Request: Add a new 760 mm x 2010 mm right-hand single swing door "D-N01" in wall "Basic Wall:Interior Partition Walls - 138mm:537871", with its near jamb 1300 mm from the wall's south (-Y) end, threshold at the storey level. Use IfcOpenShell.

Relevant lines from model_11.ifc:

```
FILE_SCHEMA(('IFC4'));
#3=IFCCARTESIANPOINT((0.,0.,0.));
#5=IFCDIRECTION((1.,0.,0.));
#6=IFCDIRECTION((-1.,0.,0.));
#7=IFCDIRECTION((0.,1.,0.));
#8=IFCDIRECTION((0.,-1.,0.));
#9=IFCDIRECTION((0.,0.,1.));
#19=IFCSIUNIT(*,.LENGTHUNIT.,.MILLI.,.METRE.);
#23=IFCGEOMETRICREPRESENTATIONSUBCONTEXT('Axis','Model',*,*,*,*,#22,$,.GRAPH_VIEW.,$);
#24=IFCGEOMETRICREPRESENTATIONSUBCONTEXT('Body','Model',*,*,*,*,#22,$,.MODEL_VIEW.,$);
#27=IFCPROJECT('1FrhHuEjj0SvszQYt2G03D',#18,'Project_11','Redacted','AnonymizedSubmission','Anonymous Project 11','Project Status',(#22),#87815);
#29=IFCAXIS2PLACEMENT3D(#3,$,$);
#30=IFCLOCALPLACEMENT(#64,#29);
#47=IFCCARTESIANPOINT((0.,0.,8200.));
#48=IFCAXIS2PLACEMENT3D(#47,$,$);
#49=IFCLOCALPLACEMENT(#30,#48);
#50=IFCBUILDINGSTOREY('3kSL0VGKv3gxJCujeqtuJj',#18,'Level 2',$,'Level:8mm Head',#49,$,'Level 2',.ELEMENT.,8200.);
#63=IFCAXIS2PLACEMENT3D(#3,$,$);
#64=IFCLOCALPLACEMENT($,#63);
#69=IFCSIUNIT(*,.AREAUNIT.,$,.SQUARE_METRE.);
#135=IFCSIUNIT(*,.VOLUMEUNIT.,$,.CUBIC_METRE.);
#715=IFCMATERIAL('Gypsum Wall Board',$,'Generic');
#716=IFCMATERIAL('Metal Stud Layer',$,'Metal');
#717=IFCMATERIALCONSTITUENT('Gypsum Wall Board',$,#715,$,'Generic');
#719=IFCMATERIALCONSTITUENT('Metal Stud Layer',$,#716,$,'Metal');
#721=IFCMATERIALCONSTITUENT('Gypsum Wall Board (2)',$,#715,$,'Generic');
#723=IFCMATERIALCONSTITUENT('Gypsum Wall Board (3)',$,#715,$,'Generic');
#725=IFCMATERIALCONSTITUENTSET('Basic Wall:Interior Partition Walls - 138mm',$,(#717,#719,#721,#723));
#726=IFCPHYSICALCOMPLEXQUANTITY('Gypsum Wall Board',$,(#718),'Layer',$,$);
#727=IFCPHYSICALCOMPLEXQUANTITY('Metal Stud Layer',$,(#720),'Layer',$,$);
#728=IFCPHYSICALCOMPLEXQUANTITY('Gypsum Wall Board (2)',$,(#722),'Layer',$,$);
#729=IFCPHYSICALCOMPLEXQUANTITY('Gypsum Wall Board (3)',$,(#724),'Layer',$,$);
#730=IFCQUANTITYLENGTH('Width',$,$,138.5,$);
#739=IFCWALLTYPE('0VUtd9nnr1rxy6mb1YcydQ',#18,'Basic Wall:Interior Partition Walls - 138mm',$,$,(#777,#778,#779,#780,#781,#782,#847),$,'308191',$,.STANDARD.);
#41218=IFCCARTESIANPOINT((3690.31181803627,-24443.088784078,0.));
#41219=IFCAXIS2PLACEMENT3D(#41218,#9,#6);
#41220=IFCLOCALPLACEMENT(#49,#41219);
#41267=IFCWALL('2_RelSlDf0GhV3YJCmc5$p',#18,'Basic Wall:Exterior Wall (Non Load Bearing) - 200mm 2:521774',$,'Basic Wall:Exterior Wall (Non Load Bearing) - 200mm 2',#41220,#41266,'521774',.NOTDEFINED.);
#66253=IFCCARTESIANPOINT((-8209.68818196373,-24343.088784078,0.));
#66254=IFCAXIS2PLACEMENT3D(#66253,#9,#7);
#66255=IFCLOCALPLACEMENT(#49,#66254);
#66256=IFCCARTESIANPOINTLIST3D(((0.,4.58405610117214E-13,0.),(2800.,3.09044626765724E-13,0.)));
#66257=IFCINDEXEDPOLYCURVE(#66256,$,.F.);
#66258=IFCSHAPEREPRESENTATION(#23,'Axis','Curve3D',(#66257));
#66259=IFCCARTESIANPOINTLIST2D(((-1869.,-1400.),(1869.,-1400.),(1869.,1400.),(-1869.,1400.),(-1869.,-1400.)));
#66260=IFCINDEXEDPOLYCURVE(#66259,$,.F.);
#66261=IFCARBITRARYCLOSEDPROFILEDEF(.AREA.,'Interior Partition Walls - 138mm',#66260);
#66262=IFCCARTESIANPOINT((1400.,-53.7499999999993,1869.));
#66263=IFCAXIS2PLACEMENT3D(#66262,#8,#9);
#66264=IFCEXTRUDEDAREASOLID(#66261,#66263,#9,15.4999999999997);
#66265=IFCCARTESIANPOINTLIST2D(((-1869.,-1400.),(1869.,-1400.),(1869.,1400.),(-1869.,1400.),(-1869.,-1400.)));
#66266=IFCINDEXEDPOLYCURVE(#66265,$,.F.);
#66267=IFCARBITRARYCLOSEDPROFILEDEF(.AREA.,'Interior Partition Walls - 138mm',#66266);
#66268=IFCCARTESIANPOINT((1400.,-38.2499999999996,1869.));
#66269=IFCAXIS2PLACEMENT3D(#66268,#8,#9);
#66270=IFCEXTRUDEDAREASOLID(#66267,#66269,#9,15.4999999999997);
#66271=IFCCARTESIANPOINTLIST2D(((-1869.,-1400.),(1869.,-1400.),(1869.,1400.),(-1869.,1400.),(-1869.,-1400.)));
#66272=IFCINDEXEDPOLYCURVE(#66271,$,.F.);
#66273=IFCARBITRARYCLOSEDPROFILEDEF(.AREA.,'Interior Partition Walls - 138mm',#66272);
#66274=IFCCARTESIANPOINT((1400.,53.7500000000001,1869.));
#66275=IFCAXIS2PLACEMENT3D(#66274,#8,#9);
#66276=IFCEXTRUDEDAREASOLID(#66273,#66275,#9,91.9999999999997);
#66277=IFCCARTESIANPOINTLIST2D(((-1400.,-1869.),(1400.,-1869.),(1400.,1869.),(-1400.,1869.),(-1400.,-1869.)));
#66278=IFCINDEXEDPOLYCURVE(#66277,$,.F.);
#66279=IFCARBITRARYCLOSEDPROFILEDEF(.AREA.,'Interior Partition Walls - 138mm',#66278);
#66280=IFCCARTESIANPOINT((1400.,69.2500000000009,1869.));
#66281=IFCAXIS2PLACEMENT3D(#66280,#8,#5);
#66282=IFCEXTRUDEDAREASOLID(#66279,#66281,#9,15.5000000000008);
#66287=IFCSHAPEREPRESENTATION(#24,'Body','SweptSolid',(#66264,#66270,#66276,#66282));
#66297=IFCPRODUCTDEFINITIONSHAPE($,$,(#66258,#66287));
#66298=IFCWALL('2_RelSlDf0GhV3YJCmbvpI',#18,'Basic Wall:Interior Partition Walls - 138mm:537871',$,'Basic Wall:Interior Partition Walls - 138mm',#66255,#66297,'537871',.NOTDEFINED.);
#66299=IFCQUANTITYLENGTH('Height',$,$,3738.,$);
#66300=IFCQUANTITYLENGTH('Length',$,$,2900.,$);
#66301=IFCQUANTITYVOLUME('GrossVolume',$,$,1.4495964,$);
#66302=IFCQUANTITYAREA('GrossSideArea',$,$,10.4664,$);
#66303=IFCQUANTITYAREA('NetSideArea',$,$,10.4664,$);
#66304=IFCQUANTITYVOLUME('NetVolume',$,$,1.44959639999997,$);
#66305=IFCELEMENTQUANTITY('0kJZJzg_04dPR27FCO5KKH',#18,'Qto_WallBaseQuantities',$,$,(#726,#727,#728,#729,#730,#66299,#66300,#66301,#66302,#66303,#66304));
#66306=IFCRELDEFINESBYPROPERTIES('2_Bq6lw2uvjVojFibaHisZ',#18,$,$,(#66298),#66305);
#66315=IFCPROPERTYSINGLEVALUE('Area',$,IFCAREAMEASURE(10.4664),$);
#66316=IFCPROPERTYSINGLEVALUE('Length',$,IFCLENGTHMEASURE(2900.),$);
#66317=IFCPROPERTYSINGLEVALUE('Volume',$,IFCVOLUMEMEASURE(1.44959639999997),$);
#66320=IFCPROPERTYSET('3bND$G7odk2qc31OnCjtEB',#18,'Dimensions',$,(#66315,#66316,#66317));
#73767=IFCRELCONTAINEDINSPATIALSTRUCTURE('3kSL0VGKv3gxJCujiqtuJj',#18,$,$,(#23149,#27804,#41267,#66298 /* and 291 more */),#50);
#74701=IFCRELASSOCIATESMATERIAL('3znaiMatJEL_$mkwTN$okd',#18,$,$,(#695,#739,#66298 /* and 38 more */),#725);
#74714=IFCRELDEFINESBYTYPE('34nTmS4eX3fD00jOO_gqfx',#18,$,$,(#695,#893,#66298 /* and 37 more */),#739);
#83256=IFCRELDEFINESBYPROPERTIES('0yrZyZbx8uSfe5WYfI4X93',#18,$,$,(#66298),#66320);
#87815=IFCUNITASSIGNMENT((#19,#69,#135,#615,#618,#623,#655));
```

```python
import numpy as np
import ifcopenshell
import ifcopenshell.api.feature
import ifcopenshell.api.geometry
import ifcopenshell.api.pset
import ifcopenshell.api.root
import ifcopenshell.api.spatial
import ifcopenshell.geom
import ifcopenshell.util.element
import ifcopenshell.util.placement
import ifcopenshell.util.representation
import ifcopenshell.util.shape
import ifcopenshell.util.unit

model = ifcopenshell.open("model_11.ifc")
unit_scale = ifcopenshell.util.unit.calculate_unit_scale(model)
area_scale = ifcopenshell.util.unit.calculate_unit_scale(model, "AREAUNIT")
volume_scale = ifcopenshell.util.unit.calculate_unit_scale(model, "VOLUMEUNIT")
settings = ifcopenshell.geom.settings()


def volume(element):
    """Net volume in cubic metres, openings subtracted."""
    shape = ifcopenshell.geom.create_shape(settings, element)
    return ifcopenshell.util.shape.get_volume(shape.geometry)


wall = model.by_guid("2_RelSlDf0GhV3YJCmbvpI")
storey = ifcopenshell.util.element.get_container(wall, ifc_class="IfcBuildingStorey")
context = ifcopenshell.util.representation.get_context(model, "Model", "Body", "MODEL_VIEW")
before = volume(wall)

width, height, from_end, sill = 0.76, 2.01, 1.3, 0.0  # metres

# The wall runs along its own X axis, and the end named is its -X end.
wall_shape = ifcopenshell.geom.create_shape(settings, wall)
x, y, z = ifcopenshell.util.shape.get_vertices(wall_shape.geometry).T
start = x.min() + from_end
face, thickness = float(y.min()), float(y.max() - y.min())
wall_matrix = ifcopenshell.util.placement.get_local_placement(wall.ObjectPlacement)
level = ifcopenshell.util.placement.get_local_placement(storey.ObjectPlacement)[2, 3]


def in_wall(x, y):
    """Placement at x, y metres in the wall's axes, at sill height."""
    matrix = wall_matrix.copy()
    matrix[:, 3] = wall_matrix @ np.array([x / unit_scale, y / unit_scale, 0.0, 1.0])
    matrix[2, 3] = level + sill / unit_scale
    return matrix


# Opening: a box that overshoots both wall faces by 50 mm.
opening = ifcopenshell.api.root.create_entity(model, ifc_class="IfcOpeningElement", predefined_type="OPENING")
box = ifcopenshell.api.geometry.add_wall_representation(
    model, context=context, length=width, height=height, thickness=thickness + 0.1
)
ifcopenshell.api.geometry.assign_representation(model, product=opening, representation=box)
ifcopenshell.api.geometry.edit_object_placement(model, product=opening, matrix=in_wall(start, face - 0.05), is_si=False)
ifcopenshell.api.feature.add_feature(model, feature=opening, element=wall)

door = ifcopenshell.api.root.create_entity(model, ifc_class="IfcDoor", name="D-N01", predefined_type="DOOR")
door.OverallWidth, door.OverallHeight = width / unit_scale, height / unit_scale
door.OperationType = "SINGLE_SWING_RIGHT"
body = ifcopenshell.api.geometry.add_door_representation(
    model,
    context=context,
    overall_width=door.OverallWidth,
    overall_height=door.OverallHeight,
    operation_type="SINGLE_SWING_RIGHT",
    lining_properties={"LiningDepth": thickness / unit_scale, "ThresholdDepth": thickness / unit_scale},
)
ifcopenshell.api.geometry.assign_representation(model, product=door, representation=body)
ifcopenshell.api.spatial.assign_container(model, products=[door], relating_structure=storey)
ifcopenshell.api.feature.add_filling(model, opening=opening, element=door)

# The lining spans the wall, so the door starts at the wall face.
ifcopenshell.api.geometry.edit_object_placement(model, product=door, matrix=in_wall(start, face), is_si=False)

after = volume(wall)

# Update the wall's stored quantities.
qto = model.by_id(ifcopenshell.util.element.get_pset(wall, "Qto_WallBaseQuantities", should_inherit=False)["id"])
ifcopenshell.api.pset.edit_qto(model, qto=qto, properties={
    "NetSideArea": after / thickness / area_scale,
    "NetVolume": after / volume_scale,
})
pset = model.by_id(ifcopenshell.util.element.get_pset(wall, "Dimensions", should_inherit=False)["id"])
ifcopenshell.api.pset.edit_pset(model, pset=pset, properties={
    "Area": model.create_entity("IfcAreaMeasure", after / thickness / area_scale),
    "Volume": model.create_entity("IfcVolumeMeasure", after / volume_scale),
})

print(f"wall volume {before:.3f} -> {after:.3f} m3")

model.write("model_11_edited.ifc")
```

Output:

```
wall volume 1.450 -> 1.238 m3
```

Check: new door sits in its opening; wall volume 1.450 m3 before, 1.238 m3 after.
